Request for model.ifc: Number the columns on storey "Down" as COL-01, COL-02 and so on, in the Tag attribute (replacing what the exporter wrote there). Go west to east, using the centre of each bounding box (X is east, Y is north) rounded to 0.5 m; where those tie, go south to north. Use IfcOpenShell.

First a look at what the model holds.

```python
import ifcopenshell
import ifcopenshell.util.element
import ifcopenshell.util.placement

model = ifcopenshell.open("model.ifc")
print(model.schema)
storey = next(s for s in model.by_type("IfcBuildingStorey") if s.Name == "Down")
columns = [e for e in ifcopenshell.util.element.get_decomposition(storey) if e.is_a("IfcColumn")]
for e in sorted(columns, key=lambda e: e.id()):
    origin = ifcopenshell.util.placement.get_local_placement(e.ObjectPlacement)[:3, 3]
    print(e.id(), e.Tag, e.Name, origin.round(2) + 0.0, sep=" | ")
```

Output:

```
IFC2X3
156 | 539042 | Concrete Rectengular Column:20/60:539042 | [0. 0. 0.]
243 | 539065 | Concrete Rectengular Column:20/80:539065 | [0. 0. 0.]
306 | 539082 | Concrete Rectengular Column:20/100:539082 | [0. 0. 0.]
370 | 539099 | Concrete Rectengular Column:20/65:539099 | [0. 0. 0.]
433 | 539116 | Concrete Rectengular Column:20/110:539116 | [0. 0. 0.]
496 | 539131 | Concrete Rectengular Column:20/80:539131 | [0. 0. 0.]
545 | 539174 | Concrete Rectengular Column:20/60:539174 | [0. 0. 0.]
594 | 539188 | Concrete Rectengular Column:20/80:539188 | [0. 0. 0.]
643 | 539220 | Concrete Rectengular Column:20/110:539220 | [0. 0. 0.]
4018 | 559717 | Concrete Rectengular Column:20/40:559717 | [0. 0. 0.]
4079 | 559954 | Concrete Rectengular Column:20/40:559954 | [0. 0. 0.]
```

```python
import ifcopenshell
import ifcopenshell.geom
import ifcopenshell.util.element
import ifcopenshell.util.shape

model = ifcopenshell.open("model.ifc")
settings = ifcopenshell.geom.settings()
settings.set("use-world-coords", True)


def centre(element):
    shape = ifcopenshell.geom.create_shape(settings, element)
    return ifcopenshell.util.shape.get_bbox_centroid(shape.geometry)


storey = next(s for s in model.by_type("IfcBuildingStorey") if s.Name == "Down")
columns = [e for e in ifcopenshell.util.element.get_decomposition(storey) if e.is_a("IfcColumn")]

# Insertion points can sit at a corner or the storey origin, so sort by the geometry (in metres).
centres = {e: centre(e) for e in columns}
columns.sort(key=lambda e: (round(centres[e][0] / 0.5), centres[e][1]))

for i, e in enumerate(columns, start=1):
    number = f"COL-{i:02d}"
    e.Tag = number
    print(e.id(), number)

model.write("model_v2.ifc")
```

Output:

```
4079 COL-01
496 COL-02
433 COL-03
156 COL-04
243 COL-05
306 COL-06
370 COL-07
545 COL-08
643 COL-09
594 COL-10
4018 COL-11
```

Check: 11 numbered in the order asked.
